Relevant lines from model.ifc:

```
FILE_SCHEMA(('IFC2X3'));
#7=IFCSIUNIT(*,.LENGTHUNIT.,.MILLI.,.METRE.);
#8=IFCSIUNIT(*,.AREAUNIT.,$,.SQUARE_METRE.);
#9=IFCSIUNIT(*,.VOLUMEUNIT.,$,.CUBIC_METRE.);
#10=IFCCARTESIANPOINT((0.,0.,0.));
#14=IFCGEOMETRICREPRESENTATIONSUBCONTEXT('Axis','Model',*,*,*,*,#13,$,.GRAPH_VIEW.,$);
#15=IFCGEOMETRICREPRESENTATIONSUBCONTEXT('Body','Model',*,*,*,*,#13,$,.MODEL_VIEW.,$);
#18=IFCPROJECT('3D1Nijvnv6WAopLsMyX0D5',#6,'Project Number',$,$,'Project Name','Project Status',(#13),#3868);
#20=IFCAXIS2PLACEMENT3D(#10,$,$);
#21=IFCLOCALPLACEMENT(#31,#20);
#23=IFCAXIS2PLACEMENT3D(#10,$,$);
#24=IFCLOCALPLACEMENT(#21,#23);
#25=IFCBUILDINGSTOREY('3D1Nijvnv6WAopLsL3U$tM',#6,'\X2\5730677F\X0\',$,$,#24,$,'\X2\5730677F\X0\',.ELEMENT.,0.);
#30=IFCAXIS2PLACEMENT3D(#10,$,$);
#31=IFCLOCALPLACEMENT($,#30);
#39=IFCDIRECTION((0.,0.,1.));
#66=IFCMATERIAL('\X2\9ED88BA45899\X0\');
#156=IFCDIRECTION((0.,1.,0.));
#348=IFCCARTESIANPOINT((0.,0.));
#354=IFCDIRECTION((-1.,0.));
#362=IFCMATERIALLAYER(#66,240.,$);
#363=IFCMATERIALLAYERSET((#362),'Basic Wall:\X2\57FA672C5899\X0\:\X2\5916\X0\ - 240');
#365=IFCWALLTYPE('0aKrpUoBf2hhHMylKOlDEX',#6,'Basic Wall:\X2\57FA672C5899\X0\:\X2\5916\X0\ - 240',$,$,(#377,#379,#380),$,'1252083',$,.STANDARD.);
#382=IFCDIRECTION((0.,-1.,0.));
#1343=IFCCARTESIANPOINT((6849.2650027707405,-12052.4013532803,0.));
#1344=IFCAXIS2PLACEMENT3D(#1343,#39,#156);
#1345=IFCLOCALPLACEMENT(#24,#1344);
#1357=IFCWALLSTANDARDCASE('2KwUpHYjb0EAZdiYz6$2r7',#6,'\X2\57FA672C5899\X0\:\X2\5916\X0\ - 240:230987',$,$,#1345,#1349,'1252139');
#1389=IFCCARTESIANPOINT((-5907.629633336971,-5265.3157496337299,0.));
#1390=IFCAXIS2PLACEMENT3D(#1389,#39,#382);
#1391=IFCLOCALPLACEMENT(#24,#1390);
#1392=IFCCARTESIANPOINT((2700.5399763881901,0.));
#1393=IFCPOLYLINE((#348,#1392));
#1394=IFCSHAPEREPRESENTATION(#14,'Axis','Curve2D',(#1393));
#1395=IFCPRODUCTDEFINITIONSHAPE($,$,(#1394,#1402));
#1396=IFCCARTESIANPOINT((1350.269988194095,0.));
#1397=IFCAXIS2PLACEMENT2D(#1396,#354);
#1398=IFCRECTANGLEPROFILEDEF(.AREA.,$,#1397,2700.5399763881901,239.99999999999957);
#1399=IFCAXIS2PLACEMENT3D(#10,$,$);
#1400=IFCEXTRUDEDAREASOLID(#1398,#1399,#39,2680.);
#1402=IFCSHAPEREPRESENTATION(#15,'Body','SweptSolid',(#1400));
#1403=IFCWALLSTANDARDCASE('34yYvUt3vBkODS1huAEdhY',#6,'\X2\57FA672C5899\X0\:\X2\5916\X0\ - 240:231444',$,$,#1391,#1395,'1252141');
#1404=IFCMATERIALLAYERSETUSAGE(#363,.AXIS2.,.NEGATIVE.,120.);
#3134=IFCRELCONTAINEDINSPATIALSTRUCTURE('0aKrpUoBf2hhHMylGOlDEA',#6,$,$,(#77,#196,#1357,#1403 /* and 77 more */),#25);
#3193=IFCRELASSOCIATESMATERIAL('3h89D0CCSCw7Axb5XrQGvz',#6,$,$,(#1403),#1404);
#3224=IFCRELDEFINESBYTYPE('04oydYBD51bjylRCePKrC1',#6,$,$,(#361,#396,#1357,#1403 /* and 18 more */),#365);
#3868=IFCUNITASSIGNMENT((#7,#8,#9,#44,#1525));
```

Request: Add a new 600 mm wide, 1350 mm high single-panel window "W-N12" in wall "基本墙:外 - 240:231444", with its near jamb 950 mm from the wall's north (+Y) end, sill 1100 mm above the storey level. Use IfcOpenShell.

```python
import numpy as np
import ifcopenshell
import ifcopenshell.api.feature
import ifcopenshell.api.geometry
import ifcopenshell.api.root
import ifcopenshell.api.spatial
import ifcopenshell.api.type
import ifcopenshell.geom
import ifcopenshell.util.element
import ifcopenshell.util.placement
import ifcopenshell.util.representation
import ifcopenshell.util.shape
import ifcopenshell.util.unit

model = ifcopenshell.open("model.ifc")
unit_scale = ifcopenshell.util.unit.calculate_unit_scale(model)
settings = ifcopenshell.geom.settings()


def volume(element):
    """Net volume in cubic metres, openings subtracted."""
    shape = ifcopenshell.geom.create_shape(settings, element)
    return ifcopenshell.util.shape.get_volume(shape.geometry)


wall = model.by_guid("34yYvUt3vBkODS1huAEdhY")
storey = ifcopenshell.util.element.get_container(wall, ifc_class="IfcBuildingStorey")
context = ifcopenshell.util.representation.get_context(model, "Model", "Body", "MODEL_VIEW")
before = volume(wall)

width, height, from_end, sill = 0.6, 1.35, 0.95, 1.1  # metres

# The wall runs along its own X axis, and the end named is its -X end.
wall_shape = ifcopenshell.geom.create_shape(settings, wall)
x, y, z = ifcopenshell.util.shape.get_vertices(wall_shape.geometry).T
start = x.min() + from_end
face, thickness = float(y.min()), float(y.max() - y.min())
wall_matrix = ifcopenshell.util.placement.get_local_placement(wall.ObjectPlacement)
level = ifcopenshell.util.placement.get_local_placement(storey.ObjectPlacement)[2, 3]


def in_wall(x, y):
    """Placement at x, y metres in the wall's axes, at sill height."""
    matrix = wall_matrix.copy()
    matrix[:, 3] = wall_matrix @ np.array([x / unit_scale, y / unit_scale, 0.0, 1.0])
    matrix[2, 3] = level + sill / unit_scale
    return matrix


# Opening: a box that overshoots both wall faces by 50 mm.
opening = ifcopenshell.api.root.create_entity(model, ifc_class="IfcOpeningElement")
box = ifcopenshell.api.geometry.add_wall_representation(
    model, context=context, length=width, height=height, thickness=thickness + 0.1
)
ifcopenshell.api.geometry.assign_representation(model, product=opening, representation=box)
ifcopenshell.api.geometry.edit_object_placement(model, product=opening, matrix=in_wall(start, face - 0.05), is_si=False)
ifcopenshell.api.feature.add_feature(model, feature=opening, element=wall)

window = ifcopenshell.api.root.create_entity(model, ifc_class="IfcWindow", name="W-N12")
window.OverallWidth, window.OverallHeight = width / unit_scale, height / unit_scale
body = ifcopenshell.api.geometry.add_window_representation(
    model,
    context=context,
    overall_width=window.OverallWidth,
    overall_height=window.OverallHeight,
    partition_type="SINGLE_PANEL",
)
ifcopenshell.api.geometry.assign_representation(model, product=window, representation=body)
ifcopenshell.api.spatial.assign_container(model, products=[window], relating_structure=storey)
fills = ifcopenshell.api.feature.add_filling(model, opening=opening, element=window)
fills.OwnerHistory = window.OwnerHistory  # required in IFC2X3

# IFC2X3 keeps the operation on the window style.
style = ifcopenshell.api.root.create_entity(model, ifc_class="IfcWindowStyle", name="W-N12")
style.OperationType, style.ConstructionType = "SINGLE_PANEL", "NOTDEFINED"
style.ParameterTakesPrecedence = style.Sizeable = False
ifcopenshell.api.type.assign_type(model, related_objects=[window], relating_type=style)

# Centre the window in the wall's thickness.
ifcopenshell.api.geometry.edit_object_placement(model, product=window, matrix=in_wall(start, face), is_si=False)
window_shape = ifcopenshell.geom.create_shape(settings, window)
depth = ifcopenshell.util.shape.get_vertices(window_shape.geometry)[:, 1]
offset = face + thickness / 2 - (depth.min() + depth.max()) / 2
ifcopenshell.api.geometry.edit_object_placement(model, product=window, matrix=in_wall(start, offset), is_si=False)

after = volume(wall)

print(f"wall volume {before:.3f} -> {after:.3f} m3")

model.write("model_rev.ifc")
```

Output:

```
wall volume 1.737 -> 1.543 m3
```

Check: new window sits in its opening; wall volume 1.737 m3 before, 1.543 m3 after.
